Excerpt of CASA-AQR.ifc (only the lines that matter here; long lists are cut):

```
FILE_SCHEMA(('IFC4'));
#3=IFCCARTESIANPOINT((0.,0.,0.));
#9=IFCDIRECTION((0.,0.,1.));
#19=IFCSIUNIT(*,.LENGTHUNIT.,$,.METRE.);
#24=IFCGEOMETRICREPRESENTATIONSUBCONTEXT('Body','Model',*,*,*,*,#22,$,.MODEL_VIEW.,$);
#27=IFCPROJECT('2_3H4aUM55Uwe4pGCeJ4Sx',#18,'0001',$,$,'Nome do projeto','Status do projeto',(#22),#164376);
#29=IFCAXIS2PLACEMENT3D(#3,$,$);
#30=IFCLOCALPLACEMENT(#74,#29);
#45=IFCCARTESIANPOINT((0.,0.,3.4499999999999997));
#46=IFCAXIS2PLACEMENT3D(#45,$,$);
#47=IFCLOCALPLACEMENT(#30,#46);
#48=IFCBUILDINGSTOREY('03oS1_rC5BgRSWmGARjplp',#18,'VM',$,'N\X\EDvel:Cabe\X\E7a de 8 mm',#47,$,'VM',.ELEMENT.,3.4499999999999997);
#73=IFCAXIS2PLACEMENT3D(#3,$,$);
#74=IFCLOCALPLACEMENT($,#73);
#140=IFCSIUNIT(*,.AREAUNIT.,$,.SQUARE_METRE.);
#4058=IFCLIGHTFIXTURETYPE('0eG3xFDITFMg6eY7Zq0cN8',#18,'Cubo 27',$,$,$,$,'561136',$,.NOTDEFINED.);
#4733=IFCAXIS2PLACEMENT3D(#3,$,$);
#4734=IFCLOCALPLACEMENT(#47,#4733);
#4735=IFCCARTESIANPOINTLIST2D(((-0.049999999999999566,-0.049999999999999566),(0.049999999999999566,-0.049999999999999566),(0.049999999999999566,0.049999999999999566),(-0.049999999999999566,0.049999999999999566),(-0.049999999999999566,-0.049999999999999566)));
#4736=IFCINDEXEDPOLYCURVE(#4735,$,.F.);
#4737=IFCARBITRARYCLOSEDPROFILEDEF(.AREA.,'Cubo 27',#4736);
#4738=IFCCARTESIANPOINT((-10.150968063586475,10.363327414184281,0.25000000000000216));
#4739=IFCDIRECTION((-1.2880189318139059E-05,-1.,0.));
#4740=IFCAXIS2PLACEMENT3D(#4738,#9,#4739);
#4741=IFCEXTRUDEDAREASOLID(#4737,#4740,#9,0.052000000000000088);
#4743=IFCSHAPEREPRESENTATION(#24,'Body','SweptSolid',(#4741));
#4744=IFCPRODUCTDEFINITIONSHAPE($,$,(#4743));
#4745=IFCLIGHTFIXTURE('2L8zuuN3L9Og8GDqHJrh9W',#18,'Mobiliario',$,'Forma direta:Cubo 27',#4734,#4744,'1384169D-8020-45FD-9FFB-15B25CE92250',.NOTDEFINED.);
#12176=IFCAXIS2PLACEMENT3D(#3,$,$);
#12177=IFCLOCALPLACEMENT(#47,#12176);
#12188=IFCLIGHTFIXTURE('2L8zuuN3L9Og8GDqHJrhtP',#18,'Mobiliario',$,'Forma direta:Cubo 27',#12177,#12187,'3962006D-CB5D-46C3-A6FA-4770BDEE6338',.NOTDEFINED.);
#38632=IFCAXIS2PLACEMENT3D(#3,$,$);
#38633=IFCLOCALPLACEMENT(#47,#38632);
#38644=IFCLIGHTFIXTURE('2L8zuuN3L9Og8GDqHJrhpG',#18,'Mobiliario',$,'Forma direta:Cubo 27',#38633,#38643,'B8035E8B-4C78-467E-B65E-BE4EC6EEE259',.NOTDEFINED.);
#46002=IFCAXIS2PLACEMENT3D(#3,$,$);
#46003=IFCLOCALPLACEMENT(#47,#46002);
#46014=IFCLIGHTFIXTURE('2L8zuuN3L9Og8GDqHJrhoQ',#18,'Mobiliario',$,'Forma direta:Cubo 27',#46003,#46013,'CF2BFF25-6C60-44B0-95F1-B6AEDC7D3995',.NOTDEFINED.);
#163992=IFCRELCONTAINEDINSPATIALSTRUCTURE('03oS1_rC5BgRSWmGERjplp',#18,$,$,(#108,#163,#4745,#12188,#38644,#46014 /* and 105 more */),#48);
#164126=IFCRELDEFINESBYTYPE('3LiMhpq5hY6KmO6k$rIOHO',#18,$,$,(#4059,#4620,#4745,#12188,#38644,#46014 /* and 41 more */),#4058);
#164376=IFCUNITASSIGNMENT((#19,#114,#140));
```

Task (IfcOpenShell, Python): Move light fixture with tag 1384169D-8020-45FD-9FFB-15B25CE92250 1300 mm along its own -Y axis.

```python
import ifcopenshell
import ifcopenshell.api.geometry
import ifcopenshell.util.placement

model = ifcopenshell.open("CASA-AQR.ifc")

item = model.by_guid("2L8zuuN3L9Og8GDqHJrh9W")
matrix = ifcopenshell.util.placement.get_local_placement(item.ObjectPlacement)
matrix[:3, 3] -= matrix[:3, 1] * 1.3
ifcopenshell.api.geometry.edit_object_placement(model, product=item, matrix=matrix, is_si=False)

print(ifcopenshell.util.placement.get_local_placement(item.ObjectPlacement).round(3) + 0.0)

model.write("CASA-AQR_updated.ifc")
```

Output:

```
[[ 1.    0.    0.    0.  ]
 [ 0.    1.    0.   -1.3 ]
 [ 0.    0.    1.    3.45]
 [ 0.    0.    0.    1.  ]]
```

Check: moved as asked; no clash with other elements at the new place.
